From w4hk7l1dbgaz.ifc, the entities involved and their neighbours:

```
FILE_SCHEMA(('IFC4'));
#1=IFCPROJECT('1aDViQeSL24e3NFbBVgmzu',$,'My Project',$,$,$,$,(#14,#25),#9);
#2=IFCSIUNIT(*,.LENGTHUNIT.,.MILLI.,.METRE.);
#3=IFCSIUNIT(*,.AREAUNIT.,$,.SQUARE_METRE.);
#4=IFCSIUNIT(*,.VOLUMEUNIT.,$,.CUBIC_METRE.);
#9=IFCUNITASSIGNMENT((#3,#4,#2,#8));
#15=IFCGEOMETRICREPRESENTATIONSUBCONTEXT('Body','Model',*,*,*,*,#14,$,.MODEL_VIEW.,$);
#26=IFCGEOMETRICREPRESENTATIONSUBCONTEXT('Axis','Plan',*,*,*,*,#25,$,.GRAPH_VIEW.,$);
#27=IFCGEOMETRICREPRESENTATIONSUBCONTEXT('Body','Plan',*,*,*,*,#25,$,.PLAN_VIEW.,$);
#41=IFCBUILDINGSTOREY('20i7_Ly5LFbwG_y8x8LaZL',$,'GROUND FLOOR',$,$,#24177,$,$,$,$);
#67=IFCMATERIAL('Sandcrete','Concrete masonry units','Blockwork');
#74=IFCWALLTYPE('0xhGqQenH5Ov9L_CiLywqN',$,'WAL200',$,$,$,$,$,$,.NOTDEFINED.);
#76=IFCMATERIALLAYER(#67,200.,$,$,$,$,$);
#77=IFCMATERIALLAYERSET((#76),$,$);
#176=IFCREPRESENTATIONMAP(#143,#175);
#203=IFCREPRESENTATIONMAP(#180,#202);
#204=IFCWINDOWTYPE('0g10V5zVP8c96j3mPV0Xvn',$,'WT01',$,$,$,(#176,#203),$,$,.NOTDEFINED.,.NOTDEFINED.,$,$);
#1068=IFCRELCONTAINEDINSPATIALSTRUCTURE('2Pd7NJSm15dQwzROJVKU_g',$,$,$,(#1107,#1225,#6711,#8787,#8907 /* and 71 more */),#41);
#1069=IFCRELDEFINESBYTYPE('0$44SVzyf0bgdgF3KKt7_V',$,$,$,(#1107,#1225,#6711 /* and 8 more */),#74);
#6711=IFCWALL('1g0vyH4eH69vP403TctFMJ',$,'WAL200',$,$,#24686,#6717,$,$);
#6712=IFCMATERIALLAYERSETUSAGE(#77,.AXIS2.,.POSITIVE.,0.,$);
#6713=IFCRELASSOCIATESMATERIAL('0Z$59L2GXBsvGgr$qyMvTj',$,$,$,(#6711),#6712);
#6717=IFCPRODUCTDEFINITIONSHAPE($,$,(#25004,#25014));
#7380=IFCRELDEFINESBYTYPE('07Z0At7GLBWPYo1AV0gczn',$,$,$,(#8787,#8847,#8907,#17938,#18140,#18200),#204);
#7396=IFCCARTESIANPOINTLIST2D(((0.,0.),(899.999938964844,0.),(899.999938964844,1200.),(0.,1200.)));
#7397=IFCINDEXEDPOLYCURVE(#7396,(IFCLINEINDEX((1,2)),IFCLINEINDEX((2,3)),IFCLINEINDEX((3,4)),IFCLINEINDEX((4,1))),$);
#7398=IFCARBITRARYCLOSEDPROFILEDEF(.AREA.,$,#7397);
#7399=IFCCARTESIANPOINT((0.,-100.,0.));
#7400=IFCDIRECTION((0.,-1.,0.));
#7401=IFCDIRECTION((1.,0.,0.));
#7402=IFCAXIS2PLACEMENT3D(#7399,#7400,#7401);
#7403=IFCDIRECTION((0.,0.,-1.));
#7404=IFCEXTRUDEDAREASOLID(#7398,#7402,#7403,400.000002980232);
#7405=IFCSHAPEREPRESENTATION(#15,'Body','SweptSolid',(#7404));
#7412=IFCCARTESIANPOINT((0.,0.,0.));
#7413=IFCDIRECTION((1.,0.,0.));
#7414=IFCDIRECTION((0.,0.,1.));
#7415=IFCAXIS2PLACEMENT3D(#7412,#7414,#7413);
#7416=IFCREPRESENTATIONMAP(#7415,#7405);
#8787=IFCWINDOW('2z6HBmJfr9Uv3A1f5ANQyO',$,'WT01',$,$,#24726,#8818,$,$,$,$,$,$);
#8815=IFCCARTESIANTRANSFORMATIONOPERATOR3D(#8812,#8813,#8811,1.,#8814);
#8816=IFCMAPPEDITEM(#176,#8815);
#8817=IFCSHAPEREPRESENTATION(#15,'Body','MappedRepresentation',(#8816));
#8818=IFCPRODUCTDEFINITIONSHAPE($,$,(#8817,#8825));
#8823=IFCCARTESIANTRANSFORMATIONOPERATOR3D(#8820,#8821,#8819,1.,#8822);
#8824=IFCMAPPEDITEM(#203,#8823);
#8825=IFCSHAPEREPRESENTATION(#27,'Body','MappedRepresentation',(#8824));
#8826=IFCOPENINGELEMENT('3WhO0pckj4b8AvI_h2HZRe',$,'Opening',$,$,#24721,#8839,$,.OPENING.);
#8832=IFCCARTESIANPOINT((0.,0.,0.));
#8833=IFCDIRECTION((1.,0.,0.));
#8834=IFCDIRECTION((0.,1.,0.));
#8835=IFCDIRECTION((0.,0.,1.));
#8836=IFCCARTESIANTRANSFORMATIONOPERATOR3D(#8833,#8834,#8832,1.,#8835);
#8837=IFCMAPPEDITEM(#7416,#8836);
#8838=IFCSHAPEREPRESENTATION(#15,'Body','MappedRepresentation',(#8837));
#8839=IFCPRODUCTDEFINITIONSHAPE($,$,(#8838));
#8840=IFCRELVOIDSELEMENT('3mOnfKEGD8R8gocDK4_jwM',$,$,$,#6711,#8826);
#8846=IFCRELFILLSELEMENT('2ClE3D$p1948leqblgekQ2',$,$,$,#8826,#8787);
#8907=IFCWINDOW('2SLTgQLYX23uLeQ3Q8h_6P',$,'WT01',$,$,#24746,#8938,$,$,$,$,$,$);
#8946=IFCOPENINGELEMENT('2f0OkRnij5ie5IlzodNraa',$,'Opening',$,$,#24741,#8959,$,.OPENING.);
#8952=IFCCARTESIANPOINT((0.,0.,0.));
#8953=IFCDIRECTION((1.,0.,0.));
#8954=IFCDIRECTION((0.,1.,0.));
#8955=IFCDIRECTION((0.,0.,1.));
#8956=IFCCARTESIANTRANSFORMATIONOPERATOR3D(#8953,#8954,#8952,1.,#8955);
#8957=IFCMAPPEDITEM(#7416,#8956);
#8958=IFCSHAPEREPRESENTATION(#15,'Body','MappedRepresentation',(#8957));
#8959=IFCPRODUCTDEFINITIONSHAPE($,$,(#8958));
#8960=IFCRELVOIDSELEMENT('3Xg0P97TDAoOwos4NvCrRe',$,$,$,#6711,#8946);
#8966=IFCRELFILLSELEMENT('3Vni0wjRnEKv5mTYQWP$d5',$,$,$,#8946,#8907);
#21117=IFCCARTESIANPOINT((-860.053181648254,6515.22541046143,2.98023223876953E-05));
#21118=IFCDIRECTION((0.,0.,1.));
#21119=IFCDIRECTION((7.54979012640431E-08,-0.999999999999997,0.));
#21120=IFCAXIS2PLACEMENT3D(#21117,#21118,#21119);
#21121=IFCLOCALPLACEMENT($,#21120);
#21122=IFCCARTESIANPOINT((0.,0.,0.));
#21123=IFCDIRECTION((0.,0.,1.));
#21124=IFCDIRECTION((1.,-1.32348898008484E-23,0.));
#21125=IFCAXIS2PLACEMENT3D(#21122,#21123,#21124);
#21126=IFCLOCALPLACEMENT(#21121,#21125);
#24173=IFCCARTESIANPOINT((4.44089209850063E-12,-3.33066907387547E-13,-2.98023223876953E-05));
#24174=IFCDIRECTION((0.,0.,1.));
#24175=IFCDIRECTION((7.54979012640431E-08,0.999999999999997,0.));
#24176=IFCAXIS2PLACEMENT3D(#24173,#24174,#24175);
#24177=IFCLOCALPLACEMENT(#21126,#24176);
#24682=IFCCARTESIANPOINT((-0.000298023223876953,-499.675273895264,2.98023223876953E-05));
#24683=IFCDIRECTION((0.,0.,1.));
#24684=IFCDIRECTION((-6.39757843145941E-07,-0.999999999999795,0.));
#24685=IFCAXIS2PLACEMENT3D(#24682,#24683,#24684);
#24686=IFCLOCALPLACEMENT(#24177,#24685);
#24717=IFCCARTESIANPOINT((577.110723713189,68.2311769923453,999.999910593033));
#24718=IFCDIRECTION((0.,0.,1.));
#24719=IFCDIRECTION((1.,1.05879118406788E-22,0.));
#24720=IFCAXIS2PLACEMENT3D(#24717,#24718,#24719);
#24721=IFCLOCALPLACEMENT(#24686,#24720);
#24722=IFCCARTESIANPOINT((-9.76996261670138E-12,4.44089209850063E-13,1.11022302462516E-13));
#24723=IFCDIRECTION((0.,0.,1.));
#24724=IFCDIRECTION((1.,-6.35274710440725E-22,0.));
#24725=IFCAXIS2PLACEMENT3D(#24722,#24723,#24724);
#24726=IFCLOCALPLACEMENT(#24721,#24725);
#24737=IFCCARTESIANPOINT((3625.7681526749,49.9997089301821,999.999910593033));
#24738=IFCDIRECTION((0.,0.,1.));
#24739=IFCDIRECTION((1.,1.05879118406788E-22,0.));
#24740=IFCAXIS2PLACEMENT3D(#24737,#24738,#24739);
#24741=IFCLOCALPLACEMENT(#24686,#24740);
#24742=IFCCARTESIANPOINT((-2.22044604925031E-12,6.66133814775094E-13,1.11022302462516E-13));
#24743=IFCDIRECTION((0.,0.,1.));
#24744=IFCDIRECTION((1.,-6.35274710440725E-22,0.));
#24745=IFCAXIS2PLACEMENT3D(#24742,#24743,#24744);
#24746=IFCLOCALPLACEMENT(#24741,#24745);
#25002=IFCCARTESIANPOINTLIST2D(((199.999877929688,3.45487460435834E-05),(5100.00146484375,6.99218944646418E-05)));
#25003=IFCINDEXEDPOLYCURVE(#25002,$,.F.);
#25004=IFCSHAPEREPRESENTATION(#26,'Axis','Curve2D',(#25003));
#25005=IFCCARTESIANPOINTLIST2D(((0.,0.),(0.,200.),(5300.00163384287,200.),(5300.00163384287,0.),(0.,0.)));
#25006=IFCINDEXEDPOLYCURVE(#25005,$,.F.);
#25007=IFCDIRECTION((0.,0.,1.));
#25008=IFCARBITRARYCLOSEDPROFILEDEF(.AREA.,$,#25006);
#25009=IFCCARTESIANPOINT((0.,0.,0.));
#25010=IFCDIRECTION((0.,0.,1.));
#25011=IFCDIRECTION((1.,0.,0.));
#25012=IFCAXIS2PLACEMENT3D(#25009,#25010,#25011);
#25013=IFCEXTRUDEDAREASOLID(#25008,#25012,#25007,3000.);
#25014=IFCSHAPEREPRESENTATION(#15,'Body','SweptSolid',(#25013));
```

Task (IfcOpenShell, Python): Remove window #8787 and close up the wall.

```python
import ifcopenshell
import ifcopenshell.api.feature
import ifcopenshell.api.root
import ifcopenshell.geom
import ifcopenshell.util.shape

model = ifcopenshell.open("w4hk7l1dbgaz.ifc")
settings = ifcopenshell.geom.settings()


def volume(element):
    """Net volume in cubic metres, openings subtracted."""
    shape = ifcopenshell.geom.create_shape(settings, element)
    return ifcopenshell.util.shape.get_volume(shape.geometry)


window = model.by_id(8787)
opening = window.FillsVoids[0].RelatingOpeningElement
wall = opening.VoidsElements[0].RelatingBuildingElement
before = volume(wall)

ifcopenshell.api.root.remove_product(model, product=window)
ifcopenshell.api.feature.remove_feature(model, feature=opening)

after = volume(wall)

print(f"wall volume {before:.3f} -> {after:.3f} m3")

model.write("w4hk7l1dbgaz_v2.ifc")
```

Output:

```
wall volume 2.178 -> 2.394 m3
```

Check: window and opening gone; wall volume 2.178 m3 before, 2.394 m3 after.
